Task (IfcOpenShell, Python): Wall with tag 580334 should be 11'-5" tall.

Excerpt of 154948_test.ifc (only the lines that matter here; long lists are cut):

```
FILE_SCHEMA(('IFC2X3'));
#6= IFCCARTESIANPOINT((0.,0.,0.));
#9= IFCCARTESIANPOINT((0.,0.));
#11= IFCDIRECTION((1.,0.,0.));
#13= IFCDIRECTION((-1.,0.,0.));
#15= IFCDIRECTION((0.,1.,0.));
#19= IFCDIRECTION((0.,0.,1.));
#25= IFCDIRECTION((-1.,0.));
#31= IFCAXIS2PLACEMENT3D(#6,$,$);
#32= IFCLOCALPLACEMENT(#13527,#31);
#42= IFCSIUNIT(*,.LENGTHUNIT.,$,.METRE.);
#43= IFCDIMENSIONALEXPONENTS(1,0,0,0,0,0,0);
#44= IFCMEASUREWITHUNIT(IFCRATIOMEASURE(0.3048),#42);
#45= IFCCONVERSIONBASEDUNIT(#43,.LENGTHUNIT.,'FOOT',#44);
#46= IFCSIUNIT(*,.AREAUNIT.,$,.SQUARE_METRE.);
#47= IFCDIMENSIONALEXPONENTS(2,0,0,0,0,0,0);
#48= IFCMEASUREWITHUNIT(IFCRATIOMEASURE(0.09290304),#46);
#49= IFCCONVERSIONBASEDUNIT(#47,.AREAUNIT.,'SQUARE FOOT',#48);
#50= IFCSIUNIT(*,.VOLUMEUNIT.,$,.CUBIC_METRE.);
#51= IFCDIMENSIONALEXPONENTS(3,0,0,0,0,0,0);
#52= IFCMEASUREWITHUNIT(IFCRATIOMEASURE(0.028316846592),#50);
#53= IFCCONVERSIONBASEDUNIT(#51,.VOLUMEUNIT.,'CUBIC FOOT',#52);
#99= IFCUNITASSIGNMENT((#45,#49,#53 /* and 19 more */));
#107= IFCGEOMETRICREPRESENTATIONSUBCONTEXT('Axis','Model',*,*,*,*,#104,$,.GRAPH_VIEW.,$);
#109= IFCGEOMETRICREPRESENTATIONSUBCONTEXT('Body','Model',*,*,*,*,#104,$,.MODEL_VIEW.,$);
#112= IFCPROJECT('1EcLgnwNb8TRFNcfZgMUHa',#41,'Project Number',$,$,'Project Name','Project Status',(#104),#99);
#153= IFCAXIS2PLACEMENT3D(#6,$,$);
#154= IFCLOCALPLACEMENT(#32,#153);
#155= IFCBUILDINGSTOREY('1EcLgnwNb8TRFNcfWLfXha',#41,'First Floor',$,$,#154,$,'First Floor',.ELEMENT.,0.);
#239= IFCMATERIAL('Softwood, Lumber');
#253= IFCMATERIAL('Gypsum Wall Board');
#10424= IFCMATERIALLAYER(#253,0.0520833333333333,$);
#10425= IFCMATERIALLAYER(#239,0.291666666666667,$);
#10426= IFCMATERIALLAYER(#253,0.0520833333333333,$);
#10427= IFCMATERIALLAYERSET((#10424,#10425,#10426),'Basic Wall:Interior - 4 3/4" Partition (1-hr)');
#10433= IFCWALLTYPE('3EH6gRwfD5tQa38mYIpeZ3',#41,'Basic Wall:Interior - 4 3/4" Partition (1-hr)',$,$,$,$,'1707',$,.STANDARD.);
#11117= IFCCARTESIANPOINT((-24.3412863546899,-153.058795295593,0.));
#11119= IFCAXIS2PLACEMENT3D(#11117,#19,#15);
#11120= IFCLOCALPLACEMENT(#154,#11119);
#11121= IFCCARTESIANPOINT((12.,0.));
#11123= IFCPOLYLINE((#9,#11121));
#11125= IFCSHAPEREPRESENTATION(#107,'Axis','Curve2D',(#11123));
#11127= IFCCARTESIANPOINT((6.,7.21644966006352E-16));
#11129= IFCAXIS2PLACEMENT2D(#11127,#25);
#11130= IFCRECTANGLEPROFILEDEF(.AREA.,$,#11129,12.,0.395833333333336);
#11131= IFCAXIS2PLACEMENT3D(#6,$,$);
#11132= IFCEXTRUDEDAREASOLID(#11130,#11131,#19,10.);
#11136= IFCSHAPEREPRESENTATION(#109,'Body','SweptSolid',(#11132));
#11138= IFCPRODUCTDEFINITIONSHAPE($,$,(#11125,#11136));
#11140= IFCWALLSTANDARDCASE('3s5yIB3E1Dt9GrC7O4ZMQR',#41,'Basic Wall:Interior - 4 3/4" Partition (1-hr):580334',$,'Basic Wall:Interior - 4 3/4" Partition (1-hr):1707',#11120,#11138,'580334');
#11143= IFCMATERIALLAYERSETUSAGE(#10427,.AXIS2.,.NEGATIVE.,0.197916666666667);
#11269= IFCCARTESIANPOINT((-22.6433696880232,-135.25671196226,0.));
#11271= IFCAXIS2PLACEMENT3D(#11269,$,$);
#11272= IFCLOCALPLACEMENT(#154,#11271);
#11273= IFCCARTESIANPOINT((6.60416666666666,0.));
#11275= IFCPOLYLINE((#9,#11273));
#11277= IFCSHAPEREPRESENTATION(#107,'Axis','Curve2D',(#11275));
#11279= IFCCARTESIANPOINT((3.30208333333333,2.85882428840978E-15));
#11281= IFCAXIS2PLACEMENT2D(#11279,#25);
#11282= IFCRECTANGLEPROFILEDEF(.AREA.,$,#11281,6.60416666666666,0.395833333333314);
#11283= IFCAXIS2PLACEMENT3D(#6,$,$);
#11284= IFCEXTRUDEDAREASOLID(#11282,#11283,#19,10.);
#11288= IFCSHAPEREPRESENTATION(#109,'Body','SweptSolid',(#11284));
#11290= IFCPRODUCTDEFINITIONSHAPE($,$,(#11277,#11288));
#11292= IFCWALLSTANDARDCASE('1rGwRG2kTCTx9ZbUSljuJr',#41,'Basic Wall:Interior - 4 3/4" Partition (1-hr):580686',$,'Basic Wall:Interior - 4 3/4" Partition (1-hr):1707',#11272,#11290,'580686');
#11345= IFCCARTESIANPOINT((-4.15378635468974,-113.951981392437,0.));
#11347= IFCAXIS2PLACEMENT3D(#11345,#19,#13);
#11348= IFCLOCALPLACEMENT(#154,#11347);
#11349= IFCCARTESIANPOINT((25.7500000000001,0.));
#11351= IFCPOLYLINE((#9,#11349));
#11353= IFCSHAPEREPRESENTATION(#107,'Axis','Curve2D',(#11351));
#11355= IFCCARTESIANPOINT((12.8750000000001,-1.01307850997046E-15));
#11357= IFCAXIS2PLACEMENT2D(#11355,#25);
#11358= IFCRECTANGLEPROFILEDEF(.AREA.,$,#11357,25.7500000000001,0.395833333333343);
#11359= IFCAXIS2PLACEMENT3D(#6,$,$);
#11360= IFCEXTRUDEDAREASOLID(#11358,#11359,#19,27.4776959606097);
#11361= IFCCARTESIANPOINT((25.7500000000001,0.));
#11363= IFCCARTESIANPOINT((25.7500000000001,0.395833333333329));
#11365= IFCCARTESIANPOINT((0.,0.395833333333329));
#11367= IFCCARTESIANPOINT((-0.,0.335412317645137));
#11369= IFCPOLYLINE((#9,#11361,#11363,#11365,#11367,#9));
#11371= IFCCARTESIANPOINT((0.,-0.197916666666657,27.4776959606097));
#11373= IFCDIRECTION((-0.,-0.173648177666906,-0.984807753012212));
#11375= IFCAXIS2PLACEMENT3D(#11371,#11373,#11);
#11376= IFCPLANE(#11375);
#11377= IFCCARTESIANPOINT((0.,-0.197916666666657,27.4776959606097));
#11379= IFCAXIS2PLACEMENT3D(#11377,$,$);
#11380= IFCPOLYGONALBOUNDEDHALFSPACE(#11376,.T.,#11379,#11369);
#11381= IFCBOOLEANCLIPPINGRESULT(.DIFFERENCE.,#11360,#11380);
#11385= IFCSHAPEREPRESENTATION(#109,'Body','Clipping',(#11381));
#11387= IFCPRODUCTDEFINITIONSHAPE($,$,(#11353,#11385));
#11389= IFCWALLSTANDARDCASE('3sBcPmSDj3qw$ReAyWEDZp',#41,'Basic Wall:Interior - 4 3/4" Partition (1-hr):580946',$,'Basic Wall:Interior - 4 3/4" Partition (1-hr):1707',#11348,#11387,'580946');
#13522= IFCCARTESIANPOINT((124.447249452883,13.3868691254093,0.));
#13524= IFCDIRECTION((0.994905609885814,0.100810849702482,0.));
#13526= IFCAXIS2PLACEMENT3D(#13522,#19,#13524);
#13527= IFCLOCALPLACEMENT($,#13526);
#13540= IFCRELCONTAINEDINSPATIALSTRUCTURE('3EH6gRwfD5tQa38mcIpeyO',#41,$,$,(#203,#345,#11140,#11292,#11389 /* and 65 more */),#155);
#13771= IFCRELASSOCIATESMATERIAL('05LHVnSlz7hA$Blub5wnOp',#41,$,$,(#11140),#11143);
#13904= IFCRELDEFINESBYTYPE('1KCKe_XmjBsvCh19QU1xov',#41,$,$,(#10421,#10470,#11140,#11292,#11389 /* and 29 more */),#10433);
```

```python
import ifcopenshell
import ifcopenshell.geom
import ifcopenshell.util.representation
import ifcopenshell.util.shape
import ifcopenshell.util.unit

model = ifcopenshell.open("154948_test.ifc")
unit_scale = ifcopenshell.util.unit.calculate_unit_scale(model)
settings = ifcopenshell.geom.settings()


def volume(element):
    """Net volume in cubic metres, openings subtracted."""
    shape = ifcopenshell.geom.create_shape(settings, element)
    return ifcopenshell.util.shape.get_volume(shape.geometry)


wall = model.by_guid("3s5yIB3E1Dt9GrC7O4ZMQR")
before = volume(wall)

body = ifcopenshell.util.representation.get_representation(wall, "Model", "Body")
solid = body.Items[0]
old_height = solid.Depth
solid.Depth = 137 * 0.0254 / unit_scale
after = volume(wall)

print(f"height {old_height:g} -> {solid.Depth:g}, volume {before:.3f} -> {after:.3f} m3")

model.write("154948_test_rev.ifc")
```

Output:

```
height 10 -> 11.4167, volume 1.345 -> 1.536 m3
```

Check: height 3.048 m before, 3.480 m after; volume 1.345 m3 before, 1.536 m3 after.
